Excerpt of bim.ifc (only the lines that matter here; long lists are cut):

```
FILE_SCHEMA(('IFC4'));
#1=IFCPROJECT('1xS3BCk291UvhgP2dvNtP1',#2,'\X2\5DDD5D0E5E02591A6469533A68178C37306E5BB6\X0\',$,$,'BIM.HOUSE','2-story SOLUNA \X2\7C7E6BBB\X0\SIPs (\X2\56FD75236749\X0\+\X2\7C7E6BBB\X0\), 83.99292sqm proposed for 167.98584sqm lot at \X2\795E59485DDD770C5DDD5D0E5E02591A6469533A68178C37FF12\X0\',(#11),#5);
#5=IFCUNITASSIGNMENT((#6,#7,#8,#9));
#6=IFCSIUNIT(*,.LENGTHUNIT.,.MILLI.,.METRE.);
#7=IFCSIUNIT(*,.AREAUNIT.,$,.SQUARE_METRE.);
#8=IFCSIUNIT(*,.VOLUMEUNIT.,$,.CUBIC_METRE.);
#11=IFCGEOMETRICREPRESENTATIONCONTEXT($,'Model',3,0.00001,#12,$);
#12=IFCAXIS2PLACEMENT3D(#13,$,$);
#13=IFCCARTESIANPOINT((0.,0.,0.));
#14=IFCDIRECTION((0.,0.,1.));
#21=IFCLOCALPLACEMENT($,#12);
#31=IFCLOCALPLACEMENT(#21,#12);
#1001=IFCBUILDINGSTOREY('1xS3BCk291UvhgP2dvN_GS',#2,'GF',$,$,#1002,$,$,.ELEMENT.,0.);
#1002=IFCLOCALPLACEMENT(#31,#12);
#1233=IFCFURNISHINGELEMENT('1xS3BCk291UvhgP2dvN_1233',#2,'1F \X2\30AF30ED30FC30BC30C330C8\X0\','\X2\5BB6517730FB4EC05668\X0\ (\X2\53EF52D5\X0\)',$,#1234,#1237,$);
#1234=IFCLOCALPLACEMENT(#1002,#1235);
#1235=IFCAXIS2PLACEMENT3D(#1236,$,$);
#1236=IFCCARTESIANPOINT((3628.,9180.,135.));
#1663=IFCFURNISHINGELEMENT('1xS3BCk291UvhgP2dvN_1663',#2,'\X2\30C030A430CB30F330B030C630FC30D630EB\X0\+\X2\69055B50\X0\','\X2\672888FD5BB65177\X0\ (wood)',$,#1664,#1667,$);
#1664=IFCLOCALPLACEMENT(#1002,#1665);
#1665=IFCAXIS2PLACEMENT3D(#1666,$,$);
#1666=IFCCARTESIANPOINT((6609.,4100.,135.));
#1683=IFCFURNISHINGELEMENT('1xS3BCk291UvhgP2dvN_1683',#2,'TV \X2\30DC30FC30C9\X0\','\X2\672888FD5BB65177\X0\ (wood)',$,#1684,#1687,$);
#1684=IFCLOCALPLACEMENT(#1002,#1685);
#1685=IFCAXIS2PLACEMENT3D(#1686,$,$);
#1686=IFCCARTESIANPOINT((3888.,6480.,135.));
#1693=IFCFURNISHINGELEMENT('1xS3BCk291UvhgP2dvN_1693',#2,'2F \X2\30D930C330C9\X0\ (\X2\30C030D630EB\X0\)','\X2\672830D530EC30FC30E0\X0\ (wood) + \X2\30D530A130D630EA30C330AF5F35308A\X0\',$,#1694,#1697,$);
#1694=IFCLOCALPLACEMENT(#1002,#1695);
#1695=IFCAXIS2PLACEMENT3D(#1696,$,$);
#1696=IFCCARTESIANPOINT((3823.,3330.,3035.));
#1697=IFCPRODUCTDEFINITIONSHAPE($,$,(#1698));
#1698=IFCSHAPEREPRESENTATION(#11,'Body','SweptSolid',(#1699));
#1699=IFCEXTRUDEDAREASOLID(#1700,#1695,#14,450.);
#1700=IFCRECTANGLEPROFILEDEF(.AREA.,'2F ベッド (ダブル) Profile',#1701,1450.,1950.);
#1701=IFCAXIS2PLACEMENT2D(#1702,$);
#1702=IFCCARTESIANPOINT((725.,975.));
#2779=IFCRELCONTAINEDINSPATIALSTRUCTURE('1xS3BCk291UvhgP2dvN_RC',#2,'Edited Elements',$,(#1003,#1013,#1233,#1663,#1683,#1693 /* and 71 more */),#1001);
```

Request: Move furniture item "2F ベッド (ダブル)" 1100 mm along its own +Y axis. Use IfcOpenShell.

```python
import ifcopenshell
import ifcopenshell.api.geometry
import ifcopenshell.util.placement

model = ifcopenshell.open("bim.ifc")

item = model.by_id(1693)
matrix = ifcopenshell.util.placement.get_local_placement(item.ObjectPlacement)
matrix[:3, 3] += matrix[:3, 1] * 1100.0
ifcopenshell.api.geometry.edit_object_placement(model, product=item, matrix=matrix, is_si=False)

print(ifcopenshell.util.placement.get_local_placement(item.ObjectPlacement).round(3) + 0.0)

model.write("bim-out.ifc")
```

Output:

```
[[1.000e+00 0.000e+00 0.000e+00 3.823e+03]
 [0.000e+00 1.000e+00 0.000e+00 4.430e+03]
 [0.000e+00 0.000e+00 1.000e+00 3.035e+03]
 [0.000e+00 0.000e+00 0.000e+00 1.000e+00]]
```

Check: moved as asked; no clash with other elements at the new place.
